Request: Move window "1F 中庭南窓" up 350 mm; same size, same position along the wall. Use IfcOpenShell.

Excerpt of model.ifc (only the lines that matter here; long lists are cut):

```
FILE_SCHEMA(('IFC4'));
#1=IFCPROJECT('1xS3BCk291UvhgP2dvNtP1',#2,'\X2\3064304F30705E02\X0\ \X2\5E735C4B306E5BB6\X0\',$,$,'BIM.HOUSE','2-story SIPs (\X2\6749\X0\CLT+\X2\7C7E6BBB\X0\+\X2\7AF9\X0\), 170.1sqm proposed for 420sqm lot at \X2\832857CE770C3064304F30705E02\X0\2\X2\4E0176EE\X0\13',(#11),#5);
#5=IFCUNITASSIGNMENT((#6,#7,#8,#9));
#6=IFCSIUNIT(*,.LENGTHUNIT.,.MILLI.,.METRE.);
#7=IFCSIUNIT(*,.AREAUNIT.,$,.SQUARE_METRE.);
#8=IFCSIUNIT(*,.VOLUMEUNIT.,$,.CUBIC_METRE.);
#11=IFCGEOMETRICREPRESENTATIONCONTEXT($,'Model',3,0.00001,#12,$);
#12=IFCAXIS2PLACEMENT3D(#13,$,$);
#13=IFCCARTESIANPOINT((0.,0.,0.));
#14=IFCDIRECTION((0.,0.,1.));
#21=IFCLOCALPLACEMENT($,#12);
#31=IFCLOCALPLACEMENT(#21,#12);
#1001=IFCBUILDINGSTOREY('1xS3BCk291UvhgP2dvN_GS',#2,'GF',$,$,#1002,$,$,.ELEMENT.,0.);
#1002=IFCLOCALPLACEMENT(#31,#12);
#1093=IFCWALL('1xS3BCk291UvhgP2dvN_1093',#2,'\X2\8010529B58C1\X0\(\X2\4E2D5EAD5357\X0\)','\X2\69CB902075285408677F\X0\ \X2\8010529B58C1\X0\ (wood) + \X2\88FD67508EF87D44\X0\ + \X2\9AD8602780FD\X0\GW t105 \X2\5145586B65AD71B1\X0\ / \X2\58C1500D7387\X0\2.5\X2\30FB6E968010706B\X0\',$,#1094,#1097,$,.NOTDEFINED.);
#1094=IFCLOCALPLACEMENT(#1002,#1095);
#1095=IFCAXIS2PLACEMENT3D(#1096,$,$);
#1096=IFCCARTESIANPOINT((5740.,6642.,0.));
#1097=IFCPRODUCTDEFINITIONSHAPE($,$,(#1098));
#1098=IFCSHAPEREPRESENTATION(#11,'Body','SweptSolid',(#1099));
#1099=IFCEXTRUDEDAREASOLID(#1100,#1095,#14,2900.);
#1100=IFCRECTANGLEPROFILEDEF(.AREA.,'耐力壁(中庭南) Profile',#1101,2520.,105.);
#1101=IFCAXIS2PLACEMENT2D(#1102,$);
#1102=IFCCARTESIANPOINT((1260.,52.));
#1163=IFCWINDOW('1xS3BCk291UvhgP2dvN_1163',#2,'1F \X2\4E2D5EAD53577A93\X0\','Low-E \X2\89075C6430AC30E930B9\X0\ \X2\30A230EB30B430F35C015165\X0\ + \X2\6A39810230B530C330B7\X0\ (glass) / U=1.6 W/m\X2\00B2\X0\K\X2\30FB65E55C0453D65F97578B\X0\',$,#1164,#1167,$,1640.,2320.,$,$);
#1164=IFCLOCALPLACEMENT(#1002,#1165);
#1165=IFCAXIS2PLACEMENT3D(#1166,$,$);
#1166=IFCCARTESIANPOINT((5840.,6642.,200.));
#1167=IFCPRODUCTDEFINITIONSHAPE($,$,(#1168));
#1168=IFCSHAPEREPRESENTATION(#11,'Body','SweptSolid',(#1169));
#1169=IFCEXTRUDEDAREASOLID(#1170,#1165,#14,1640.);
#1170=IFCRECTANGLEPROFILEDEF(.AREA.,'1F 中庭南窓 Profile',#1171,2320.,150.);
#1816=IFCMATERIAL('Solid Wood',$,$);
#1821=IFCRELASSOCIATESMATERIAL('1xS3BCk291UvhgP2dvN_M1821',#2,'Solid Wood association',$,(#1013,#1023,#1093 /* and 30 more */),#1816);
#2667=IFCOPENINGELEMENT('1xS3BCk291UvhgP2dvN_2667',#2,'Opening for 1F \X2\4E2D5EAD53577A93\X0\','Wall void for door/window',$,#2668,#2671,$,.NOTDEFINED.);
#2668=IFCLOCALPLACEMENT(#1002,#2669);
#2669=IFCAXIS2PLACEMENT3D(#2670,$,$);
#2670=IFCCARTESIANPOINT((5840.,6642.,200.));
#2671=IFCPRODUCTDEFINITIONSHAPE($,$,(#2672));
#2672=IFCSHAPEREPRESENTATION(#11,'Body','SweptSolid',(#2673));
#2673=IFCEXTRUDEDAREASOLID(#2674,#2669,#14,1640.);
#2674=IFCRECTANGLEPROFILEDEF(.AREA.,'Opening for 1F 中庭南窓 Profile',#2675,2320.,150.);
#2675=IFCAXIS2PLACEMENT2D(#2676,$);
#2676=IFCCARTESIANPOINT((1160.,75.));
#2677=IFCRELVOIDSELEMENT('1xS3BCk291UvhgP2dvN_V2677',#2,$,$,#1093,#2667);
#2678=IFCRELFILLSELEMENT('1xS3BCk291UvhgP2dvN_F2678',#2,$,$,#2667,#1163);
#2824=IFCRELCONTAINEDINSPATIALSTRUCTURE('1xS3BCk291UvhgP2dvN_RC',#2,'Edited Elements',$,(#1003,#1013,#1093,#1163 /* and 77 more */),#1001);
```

```python
import numpy as np
import ifcopenshell
import ifcopenshell.api.geometry
import ifcopenshell.util.placement
import ifcopenshell.util.unit

model = ifcopenshell.open("model.ifc")
unit_scale = ifcopenshell.util.unit.calculate_unit_scale(model)

window = model.by_guid("1xS3BCk291UvhgP2dvN_1163")
opening = window.FillsVoids[0].RelatingOpeningElement
dz = 0.35 / unit_scale

shift = np.array([0.0, 0.0, dz])
# The window is not placed relative to its opening, so move both.
for product in (opening, window):
    matrix = ifcopenshell.util.placement.get_local_placement(product.ObjectPlacement)
    matrix[:3, 3] += shift
    ifcopenshell.api.geometry.edit_object_placement(model, product=product, matrix=matrix, is_si=False)

print(f"moved by {dz * unit_scale:+.3f} m")

model.write("model-out.ifc")
```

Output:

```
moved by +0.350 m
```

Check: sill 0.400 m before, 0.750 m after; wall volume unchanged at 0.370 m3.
